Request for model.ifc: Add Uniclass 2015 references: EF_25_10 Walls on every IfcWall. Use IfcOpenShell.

First a look at what the model holds.

```python
import ifcopenshell

model = ifcopenshell.open("model.ifc")
print(model.schema)
print("classifications:", [c.Name for c in model.by_type("IfcClassification")])
for ifc_class in ("IfcDoor", "IfcRoof", "IfcStair", "IfcWall", "IfcWindow"):
    print(ifc_class, len(model.by_type(ifc_class)))
```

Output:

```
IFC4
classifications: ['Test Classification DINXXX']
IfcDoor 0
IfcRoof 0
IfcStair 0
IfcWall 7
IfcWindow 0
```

```python
import ifcopenshell
import ifcopenshell.api.classification

model = ifcopenshell.open("model.ifc")

system = ifcopenshell.api.classification.add_classification(model, classification="Uniclass 2015")

codes = {
    "IfcWall": ("EF_25_10", "Walls"),
}
for ifc_class, (code, name) in codes.items():
    products = model.by_type(ifc_class)
    ifcopenshell.api.classification.add_reference(
        model, products=products, classification=system, identification=code, name=name
    )
    print(code, len(products))

model.write("model-out.ifc")
```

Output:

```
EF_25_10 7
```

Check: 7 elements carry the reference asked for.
